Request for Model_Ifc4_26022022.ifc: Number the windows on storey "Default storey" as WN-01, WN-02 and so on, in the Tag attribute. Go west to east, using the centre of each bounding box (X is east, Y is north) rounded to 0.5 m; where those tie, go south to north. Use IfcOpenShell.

First a look at what the model holds.

```python
import ifcopenshell
import ifcopenshell.util.element
import ifcopenshell.util.placement

model = ifcopenshell.open("Model_Ifc4_26022022.ifc")
print(model.schema)
storey = next(s for s in model.by_type("IfcBuildingStorey") if s.Name == "Default storey")
windows = [e for e in ifcopenshell.util.element.get_decomposition(storey) if e.is_a("IfcWindow")]
for e in sorted(windows, key=lambda e: e.id()):
    origin = ifcopenshell.util.placement.get_local_placement(e.ObjectPlacement)[:3, 3]
    print(e.id(), e.Tag, e.Name, origin.round(2) + 0.0, sep=" | ")
```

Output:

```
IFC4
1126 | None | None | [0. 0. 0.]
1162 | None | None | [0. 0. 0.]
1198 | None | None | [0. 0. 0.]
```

```python
import ifcopenshell
import ifcopenshell.geom
import ifcopenshell.util.element
import ifcopenshell.util.shape

model = ifcopenshell.open("Model_Ifc4_26022022.ifc")
settings = ifcopenshell.geom.settings()
settings.set("use-world-coords", True)


def centre(element):
    shape = ifcopenshell.geom.create_shape(settings, element)
    return ifcopenshell.util.shape.get_bbox_centroid(shape.geometry)


storey = next(s for s in model.by_type("IfcBuildingStorey") if s.Name == "Default storey")
windows = [e for e in ifcopenshell.util.element.get_decomposition(storey) if e.is_a("IfcWindow")]

# Insertion points can sit at a corner or the storey origin, so sort by the geometry (in metres).
centres = {e: centre(e) for e in windows}
windows.sort(key=lambda e: (round(centres[e][0] / 0.5), centres[e][1]))

for i, e in enumerate(windows, start=1):
    number = f"WN-{i:02d}"
    e.Tag = number
    print(e.id(), number)

model.write("Model_Ifc4_26022022-out.ifc")
```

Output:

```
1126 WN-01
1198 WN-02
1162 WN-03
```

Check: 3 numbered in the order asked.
